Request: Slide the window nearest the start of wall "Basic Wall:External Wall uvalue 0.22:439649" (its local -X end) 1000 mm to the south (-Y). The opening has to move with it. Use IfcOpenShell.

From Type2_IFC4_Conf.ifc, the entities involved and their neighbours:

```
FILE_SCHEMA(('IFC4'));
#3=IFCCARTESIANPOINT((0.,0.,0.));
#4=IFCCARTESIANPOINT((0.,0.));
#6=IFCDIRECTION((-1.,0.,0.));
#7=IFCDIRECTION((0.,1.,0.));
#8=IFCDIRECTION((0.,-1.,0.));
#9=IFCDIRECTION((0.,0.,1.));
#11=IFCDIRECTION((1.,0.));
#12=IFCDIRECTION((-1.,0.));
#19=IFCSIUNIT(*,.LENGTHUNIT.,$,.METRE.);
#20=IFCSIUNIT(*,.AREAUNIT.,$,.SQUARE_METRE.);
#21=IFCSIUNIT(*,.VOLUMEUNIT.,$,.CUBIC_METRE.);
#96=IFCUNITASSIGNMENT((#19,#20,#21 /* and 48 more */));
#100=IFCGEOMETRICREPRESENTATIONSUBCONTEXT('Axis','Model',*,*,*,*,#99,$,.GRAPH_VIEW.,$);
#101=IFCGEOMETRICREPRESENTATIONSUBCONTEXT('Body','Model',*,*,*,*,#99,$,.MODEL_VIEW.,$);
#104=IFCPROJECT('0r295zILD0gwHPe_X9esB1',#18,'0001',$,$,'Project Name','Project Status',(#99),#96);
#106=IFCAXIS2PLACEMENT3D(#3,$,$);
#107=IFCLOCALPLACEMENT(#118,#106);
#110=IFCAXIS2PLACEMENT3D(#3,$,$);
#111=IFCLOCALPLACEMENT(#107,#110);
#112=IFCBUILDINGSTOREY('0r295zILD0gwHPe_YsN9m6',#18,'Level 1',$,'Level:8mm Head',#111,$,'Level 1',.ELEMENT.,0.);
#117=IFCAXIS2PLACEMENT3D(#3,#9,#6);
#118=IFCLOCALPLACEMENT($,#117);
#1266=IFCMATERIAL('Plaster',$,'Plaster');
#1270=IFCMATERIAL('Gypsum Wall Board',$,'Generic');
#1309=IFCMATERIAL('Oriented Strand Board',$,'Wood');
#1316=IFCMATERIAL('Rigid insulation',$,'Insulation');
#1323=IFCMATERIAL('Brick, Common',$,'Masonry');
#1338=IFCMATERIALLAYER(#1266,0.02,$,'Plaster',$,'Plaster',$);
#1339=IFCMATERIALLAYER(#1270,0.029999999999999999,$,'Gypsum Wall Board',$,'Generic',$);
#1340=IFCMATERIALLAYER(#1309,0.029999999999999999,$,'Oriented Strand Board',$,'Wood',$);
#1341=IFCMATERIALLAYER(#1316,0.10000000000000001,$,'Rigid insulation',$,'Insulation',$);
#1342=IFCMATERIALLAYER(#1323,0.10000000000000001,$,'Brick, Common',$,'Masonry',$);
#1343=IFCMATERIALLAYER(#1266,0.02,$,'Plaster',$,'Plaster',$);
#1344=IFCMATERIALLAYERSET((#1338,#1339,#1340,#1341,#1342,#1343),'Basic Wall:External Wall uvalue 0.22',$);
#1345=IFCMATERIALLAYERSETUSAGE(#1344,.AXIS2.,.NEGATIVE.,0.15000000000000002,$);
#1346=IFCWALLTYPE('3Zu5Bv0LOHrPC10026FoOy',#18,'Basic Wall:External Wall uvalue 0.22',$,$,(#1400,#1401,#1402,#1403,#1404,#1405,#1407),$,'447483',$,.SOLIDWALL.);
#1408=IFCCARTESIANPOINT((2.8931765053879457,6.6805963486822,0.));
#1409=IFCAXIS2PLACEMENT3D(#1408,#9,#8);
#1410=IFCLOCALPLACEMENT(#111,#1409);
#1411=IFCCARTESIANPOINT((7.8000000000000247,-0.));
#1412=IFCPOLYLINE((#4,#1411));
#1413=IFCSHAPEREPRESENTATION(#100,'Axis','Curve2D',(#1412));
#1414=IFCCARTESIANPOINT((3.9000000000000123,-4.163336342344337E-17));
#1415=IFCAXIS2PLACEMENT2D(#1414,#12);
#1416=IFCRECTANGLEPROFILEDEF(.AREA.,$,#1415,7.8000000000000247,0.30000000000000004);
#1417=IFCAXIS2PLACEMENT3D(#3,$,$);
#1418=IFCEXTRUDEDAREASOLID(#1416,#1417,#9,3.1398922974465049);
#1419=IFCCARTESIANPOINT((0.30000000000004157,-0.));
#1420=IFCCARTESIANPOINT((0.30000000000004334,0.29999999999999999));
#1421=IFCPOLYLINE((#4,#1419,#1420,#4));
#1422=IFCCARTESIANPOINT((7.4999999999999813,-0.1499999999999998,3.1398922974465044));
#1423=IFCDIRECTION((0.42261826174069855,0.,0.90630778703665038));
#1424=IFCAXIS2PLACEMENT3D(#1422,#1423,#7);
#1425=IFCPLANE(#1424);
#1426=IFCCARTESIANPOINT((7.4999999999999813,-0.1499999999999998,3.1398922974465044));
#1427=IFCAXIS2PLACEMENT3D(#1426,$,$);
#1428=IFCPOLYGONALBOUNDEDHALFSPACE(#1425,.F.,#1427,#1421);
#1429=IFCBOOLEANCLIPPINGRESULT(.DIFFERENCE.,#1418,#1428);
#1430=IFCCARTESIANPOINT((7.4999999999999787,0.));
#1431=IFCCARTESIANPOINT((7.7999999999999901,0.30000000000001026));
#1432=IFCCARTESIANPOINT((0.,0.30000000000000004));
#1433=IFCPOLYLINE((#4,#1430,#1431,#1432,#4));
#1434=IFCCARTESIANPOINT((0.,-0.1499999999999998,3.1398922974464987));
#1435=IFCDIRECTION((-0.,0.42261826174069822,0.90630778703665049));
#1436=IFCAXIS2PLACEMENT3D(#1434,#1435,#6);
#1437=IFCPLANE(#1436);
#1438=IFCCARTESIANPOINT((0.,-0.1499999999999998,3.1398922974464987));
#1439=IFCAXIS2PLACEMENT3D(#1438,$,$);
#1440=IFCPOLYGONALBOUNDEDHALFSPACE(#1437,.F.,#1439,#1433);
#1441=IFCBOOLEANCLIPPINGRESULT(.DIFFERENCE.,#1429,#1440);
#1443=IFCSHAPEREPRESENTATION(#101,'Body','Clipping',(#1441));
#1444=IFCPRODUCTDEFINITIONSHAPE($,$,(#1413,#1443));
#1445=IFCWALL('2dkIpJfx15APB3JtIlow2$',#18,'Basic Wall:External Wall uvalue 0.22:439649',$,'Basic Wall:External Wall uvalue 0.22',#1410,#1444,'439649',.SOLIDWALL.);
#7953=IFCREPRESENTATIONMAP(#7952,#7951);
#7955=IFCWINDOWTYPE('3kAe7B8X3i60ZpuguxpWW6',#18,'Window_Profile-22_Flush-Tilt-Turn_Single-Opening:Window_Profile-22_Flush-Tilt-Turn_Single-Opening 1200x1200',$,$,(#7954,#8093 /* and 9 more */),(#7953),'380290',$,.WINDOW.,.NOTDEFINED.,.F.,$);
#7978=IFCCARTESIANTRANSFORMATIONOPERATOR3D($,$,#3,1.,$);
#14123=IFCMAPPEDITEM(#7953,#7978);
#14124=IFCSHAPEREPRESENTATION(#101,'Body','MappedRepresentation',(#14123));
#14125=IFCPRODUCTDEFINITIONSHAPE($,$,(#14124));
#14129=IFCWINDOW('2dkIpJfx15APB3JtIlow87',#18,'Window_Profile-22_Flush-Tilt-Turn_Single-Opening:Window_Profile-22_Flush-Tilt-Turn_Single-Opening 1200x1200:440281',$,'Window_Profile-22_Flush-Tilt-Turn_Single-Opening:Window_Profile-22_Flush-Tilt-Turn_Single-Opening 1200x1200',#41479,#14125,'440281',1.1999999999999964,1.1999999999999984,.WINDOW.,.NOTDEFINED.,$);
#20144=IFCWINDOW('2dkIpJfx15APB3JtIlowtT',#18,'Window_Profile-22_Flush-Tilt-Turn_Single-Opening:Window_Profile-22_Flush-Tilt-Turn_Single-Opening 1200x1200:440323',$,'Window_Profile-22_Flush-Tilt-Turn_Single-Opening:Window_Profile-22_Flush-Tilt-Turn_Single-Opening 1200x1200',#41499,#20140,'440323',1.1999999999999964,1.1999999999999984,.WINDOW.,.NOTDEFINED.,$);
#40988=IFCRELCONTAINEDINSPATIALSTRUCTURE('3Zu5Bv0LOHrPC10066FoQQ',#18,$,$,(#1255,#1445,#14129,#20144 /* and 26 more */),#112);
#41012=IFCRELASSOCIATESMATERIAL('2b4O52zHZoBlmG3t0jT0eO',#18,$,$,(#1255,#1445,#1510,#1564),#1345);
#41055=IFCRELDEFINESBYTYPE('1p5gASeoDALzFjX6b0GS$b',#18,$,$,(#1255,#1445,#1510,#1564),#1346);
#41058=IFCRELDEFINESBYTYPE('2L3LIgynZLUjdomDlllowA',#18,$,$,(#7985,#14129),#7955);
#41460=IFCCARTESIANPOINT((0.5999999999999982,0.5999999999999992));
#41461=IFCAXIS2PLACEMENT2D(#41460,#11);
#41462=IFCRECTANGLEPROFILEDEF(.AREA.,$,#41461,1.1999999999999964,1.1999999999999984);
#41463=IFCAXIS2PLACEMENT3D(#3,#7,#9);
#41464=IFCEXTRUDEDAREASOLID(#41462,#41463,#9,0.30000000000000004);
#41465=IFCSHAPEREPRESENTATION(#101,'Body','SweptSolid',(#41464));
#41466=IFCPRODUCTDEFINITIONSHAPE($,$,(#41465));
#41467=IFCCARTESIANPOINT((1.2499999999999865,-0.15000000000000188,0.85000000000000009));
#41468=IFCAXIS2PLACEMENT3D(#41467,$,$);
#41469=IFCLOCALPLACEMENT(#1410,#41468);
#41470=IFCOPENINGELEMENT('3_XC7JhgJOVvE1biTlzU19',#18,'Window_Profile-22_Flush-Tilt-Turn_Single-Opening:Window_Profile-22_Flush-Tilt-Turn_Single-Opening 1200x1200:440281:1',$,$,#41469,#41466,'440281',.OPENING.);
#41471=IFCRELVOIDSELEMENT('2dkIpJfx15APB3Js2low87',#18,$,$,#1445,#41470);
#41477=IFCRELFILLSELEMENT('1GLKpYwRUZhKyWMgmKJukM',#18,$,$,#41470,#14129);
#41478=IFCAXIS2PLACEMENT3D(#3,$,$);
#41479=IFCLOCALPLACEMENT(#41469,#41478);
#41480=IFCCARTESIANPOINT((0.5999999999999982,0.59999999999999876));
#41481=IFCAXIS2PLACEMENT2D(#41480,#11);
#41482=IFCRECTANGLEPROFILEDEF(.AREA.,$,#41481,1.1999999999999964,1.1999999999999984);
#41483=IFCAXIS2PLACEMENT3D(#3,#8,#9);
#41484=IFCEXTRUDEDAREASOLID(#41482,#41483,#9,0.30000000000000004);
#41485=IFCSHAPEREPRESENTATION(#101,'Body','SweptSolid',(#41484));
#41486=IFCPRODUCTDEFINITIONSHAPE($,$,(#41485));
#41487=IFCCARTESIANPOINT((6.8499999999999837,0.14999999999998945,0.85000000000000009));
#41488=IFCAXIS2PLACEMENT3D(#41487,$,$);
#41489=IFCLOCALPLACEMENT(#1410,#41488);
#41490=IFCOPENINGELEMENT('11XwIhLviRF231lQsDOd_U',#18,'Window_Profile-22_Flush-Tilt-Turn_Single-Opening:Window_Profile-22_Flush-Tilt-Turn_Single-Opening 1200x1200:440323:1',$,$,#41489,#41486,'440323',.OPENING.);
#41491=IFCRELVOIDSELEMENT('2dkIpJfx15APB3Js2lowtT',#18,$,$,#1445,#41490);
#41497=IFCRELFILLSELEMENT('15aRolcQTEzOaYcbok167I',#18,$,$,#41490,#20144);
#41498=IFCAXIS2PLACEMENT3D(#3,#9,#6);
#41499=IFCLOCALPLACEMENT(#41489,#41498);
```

```python
import ifcopenshell
import ifcopenshell.api.geometry
import ifcopenshell.util.placement

model = ifcopenshell.open("Type2_IFC4_Conf.ifc")

window = model.by_guid("2dkIpJfx15APB3JtIlow87")
opening = window.FillsVoids[0].RelatingOpeningElement
wall = opening.VoidsElements[0].RelatingBuildingElement

wall_matrix = ifcopenshell.util.placement.get_local_placement(wall.ObjectPlacement)
shift = wall_matrix[:3, 0] * -1.0
before = ifcopenshell.util.placement.get_local_placement(window.ObjectPlacement)[:3, 3].copy()

# The window is placed relative to its opening, so it follows when the opening moves.
matrix = ifcopenshell.util.placement.get_local_placement(opening.ObjectPlacement)
matrix[:3, 3] += shift
ifcopenshell.api.geometry.edit_object_placement(
    model, product=opening, matrix=matrix, is_si=False, should_transform_children=True
)

after = ifcopenshell.util.placement.get_local_placement(window.ObjectPlacement)[:3, 3]
print("window moved by", (after - before).round(3) + 0.0)

model.write("Type2_IFC4_Conf_rev.ifc")
```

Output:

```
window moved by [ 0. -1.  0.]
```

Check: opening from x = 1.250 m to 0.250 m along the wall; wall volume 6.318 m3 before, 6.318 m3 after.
